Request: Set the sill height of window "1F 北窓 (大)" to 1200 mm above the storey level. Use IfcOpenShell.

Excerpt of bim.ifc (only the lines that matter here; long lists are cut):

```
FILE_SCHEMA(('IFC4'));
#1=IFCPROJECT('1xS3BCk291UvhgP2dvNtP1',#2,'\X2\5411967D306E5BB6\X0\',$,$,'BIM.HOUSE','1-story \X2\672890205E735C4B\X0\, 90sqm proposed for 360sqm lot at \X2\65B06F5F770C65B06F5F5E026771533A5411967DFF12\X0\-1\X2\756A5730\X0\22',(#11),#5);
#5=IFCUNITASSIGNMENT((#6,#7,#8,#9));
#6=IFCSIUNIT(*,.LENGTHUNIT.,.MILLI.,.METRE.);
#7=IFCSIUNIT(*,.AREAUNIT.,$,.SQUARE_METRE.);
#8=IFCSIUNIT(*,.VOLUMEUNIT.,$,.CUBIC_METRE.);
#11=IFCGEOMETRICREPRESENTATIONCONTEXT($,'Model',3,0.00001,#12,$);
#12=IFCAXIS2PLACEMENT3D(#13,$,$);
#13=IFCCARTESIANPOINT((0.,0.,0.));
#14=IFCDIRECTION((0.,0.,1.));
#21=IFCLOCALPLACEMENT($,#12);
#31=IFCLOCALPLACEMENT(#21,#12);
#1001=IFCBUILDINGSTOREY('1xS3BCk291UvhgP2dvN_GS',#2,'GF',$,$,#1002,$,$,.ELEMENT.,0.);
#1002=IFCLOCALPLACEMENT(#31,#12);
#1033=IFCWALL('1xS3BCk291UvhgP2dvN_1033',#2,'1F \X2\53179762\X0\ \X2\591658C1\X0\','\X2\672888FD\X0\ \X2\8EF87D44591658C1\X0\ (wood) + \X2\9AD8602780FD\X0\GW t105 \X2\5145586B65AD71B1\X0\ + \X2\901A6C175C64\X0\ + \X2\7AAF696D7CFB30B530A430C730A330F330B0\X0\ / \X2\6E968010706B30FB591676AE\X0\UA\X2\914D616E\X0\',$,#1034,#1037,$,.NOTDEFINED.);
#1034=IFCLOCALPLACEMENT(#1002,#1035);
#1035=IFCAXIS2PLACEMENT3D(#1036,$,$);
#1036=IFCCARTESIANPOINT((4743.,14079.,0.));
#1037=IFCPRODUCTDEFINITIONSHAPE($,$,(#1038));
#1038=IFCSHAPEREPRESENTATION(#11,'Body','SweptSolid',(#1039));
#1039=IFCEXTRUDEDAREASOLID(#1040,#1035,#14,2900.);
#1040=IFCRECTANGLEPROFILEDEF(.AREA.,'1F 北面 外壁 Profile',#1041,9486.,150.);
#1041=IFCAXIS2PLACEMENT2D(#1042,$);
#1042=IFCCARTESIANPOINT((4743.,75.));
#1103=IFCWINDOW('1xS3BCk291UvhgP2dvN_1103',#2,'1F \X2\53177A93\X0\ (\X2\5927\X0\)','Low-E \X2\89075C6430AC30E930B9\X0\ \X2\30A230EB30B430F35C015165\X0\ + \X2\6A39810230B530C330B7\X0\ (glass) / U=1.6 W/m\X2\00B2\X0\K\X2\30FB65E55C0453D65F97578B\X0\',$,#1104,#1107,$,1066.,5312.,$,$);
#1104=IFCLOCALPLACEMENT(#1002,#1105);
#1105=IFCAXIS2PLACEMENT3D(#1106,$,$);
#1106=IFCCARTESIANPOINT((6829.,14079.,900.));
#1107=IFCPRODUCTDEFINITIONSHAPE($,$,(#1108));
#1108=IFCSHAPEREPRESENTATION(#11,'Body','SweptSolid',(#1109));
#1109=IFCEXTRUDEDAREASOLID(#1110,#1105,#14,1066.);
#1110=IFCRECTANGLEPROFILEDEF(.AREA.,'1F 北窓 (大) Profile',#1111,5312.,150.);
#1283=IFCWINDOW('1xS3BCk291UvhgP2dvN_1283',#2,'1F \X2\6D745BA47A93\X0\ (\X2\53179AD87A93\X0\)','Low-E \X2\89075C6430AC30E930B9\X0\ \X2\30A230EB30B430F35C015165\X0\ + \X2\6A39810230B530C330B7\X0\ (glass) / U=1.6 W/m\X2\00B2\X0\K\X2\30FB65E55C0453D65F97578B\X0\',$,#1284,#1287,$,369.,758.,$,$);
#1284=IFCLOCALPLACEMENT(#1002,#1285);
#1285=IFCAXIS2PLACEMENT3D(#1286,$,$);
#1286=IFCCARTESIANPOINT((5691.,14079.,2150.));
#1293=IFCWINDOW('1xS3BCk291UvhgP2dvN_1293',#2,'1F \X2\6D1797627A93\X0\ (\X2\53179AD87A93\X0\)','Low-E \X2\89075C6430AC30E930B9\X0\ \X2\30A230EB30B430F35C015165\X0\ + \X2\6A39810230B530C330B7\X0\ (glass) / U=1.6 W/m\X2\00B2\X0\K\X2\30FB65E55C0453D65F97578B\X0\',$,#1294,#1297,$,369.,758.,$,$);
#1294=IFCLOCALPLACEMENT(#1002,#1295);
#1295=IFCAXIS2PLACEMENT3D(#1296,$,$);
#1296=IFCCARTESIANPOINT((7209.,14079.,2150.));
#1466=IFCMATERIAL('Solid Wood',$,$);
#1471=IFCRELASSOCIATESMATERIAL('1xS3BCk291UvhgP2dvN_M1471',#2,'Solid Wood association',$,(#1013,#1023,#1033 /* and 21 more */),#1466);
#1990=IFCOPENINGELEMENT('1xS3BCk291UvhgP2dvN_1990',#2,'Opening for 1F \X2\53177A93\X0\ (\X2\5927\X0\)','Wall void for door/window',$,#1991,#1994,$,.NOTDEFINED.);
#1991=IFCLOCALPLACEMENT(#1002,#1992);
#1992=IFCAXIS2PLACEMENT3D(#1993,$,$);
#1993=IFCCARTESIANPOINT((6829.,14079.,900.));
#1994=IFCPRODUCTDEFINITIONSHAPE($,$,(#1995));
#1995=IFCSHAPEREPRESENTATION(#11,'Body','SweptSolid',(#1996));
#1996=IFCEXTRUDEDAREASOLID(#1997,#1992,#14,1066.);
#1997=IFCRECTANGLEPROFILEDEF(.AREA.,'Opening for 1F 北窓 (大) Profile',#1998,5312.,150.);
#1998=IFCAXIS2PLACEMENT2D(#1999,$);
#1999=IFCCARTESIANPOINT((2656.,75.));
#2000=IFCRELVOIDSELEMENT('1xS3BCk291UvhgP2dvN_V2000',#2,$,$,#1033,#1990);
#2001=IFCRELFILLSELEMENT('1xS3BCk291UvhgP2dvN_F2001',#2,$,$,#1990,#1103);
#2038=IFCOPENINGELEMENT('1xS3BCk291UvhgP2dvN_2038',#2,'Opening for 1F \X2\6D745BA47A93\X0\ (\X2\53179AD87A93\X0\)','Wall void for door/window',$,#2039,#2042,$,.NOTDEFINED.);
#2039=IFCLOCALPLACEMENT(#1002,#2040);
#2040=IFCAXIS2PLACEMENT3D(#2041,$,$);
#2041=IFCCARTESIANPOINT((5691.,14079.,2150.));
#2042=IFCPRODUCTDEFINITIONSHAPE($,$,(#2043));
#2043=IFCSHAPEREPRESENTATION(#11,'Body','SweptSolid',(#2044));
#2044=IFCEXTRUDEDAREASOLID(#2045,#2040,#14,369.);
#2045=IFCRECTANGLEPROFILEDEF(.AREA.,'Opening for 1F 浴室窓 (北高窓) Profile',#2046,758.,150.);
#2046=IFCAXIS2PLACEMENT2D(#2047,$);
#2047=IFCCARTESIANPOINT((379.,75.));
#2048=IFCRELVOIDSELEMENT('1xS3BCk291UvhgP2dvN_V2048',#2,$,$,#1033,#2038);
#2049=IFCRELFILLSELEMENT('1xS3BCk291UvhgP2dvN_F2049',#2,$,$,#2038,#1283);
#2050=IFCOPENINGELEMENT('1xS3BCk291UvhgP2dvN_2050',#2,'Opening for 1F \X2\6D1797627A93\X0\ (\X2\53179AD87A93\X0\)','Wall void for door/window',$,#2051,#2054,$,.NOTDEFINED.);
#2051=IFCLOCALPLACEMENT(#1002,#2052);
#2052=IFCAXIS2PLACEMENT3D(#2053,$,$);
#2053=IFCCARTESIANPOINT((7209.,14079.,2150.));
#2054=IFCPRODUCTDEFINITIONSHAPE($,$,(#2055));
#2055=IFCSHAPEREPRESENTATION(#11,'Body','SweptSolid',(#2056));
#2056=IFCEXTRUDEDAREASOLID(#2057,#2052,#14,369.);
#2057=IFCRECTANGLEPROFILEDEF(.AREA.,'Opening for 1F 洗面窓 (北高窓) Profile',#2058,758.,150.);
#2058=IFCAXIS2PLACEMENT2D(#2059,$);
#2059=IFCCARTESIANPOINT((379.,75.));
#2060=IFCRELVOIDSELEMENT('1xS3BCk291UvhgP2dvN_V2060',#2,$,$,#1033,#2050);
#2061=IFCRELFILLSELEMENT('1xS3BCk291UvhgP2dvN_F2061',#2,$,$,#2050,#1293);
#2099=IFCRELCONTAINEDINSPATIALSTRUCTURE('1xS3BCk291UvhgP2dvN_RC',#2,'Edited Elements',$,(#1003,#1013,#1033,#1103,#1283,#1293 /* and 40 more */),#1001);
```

```python
import numpy as np
import ifcopenshell
import ifcopenshell.api.geometry
import ifcopenshell.geom
import ifcopenshell.util.element
import ifcopenshell.util.placement
import ifcopenshell.util.shape
import ifcopenshell.util.unit

model = ifcopenshell.open("bim.ifc")
unit_scale = ifcopenshell.util.unit.calculate_unit_scale(model)

window = model.by_guid("1xS3BCk291UvhgP2dvN_1103")
opening = window.FillsVoids[0].RelatingOpeningElement
storey = ifcopenshell.util.element.get_container(window, ifc_class="IfcBuildingStorey")
level = ifcopenshell.util.placement.get_local_placement(storey.ObjectPlacement)[2, 3]

# The opening's origin need not be at the sill, so measure its lowest point.
shape = ifcopenshell.geom.create_shape(ifcopenshell.geom.settings(), opening)
bottom = ifcopenshell.util.shape.get_shape_bottom_elevation(shape, shape.geometry) / unit_scale
dz = level + 1.2 / unit_scale - bottom

shift = np.array([0.0, 0.0, dz])
# The window is not placed relative to its opening, so move both.
for product in (opening, window):
    matrix = ifcopenshell.util.placement.get_local_placement(product.ObjectPlacement)
    matrix[:3, 3] += shift
    ifcopenshell.api.geometry.edit_object_placement(model, product=product, matrix=matrix, is_si=False)

print(f"moved by {dz * unit_scale:+.3f} m")

model.write("bim_v2.ifc")
```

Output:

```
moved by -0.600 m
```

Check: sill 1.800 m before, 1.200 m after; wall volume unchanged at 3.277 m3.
